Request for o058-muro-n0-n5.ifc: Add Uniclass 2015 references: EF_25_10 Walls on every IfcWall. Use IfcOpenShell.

First a look at what the model holds.

```python
import ifcopenshell

model = ifcopenshell.open("o058-muro-n0-n5.ifc")
print(model.schema)
print("classifications:", [c.Name for c in model.by_type("IfcClassification")])
for ifc_class in ("IfcDoor", "IfcRoof", "IfcStair", "IfcWall", "IfcWindow"):
    print(ifc_class, len(model.by_type(ifc_class)))
```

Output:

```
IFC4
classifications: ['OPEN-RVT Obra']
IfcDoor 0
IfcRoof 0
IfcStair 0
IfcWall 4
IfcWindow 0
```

```python
import ifcopenshell
import ifcopenshell.api.classification

model = ifcopenshell.open("o058-muro-n0-n5.ifc")

system = ifcopenshell.api.classification.add_classification(model, classification="Uniclass 2015")

codes = {
    "IfcWall": ("EF_25_10", "Walls"),
}
for ifc_class, (code, name) in codes.items():
    products = model.by_type(ifc_class)
    ifcopenshell.api.classification.add_reference(
        model, products=products, classification=system, identification=code, name=name
    )
    print(code, len(products))

model.write("o058-muro-n0-n5-out.ifc")
```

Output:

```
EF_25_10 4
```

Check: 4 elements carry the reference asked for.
